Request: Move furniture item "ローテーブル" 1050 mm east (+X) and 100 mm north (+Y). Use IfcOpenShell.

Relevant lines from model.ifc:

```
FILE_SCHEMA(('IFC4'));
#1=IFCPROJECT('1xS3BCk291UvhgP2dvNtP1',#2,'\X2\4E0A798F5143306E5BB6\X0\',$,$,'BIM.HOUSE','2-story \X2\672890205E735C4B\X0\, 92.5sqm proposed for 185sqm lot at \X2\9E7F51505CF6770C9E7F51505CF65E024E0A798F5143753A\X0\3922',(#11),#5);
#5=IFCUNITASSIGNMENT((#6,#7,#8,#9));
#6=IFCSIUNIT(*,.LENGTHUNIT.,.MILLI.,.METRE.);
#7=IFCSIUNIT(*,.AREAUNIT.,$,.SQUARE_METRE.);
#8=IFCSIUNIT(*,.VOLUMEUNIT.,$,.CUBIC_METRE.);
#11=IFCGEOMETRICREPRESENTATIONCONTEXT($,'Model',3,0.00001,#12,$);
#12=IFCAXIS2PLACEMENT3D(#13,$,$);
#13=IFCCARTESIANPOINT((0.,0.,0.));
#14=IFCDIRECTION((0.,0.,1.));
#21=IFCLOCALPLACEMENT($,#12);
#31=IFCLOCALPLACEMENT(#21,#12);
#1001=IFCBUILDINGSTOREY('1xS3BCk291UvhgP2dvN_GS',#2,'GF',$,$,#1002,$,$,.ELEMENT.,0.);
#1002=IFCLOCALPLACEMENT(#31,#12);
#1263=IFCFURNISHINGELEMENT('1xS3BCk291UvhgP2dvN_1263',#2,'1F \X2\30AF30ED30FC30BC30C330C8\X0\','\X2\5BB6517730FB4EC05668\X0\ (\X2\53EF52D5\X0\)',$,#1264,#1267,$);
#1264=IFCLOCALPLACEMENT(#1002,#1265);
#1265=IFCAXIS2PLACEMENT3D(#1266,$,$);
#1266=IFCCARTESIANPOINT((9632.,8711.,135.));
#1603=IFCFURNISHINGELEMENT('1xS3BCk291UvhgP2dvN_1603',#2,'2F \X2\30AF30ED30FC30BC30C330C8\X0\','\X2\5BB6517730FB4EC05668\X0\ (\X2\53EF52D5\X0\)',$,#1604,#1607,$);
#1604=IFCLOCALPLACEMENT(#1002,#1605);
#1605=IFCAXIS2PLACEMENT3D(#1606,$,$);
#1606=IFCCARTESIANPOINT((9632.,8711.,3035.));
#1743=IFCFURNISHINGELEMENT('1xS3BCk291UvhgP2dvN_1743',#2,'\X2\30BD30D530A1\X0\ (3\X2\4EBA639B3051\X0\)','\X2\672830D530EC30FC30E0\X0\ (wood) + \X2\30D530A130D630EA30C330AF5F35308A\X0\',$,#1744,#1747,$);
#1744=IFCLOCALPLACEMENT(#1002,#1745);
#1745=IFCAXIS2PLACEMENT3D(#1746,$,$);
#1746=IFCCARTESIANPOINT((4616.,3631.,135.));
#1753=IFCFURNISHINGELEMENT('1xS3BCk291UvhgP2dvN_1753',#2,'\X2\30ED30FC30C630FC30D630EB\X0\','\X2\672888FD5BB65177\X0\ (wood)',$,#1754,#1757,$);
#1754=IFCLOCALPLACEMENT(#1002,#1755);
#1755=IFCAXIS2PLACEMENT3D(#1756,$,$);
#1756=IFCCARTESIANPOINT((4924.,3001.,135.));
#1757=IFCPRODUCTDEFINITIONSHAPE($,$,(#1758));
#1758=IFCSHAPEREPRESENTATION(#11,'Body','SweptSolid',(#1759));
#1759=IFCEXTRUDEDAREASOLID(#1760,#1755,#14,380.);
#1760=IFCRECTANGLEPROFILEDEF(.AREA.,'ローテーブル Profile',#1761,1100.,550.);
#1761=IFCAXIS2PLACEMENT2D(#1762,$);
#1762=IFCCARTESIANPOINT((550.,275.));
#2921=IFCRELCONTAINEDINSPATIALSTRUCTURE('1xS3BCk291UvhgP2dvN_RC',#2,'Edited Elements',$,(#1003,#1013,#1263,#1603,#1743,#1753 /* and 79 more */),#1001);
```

```python
import ifcopenshell
import ifcopenshell.api.geometry
import ifcopenshell.util.placement
import ifcopenshell.util.unit

model = ifcopenshell.open("model.ifc")
unit_scale = ifcopenshell.util.unit.calculate_unit_scale(model)

item = model.by_guid("1xS3BCk291UvhgP2dvN_1753")
matrix = ifcopenshell.util.placement.get_local_placement(item.ObjectPlacement)
matrix[0, 3] += 1.05 / unit_scale
matrix[1, 3] += 0.1 / unit_scale
ifcopenshell.api.geometry.edit_object_placement(model, product=item, matrix=matrix, is_si=False)

print(ifcopenshell.util.placement.get_local_placement(item.ObjectPlacement).round(3) + 0.0)

model.write("model_v2.ifc")
```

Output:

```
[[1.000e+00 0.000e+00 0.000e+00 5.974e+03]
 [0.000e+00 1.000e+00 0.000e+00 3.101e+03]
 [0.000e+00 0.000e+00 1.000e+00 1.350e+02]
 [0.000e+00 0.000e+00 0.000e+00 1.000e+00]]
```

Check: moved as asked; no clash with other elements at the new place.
